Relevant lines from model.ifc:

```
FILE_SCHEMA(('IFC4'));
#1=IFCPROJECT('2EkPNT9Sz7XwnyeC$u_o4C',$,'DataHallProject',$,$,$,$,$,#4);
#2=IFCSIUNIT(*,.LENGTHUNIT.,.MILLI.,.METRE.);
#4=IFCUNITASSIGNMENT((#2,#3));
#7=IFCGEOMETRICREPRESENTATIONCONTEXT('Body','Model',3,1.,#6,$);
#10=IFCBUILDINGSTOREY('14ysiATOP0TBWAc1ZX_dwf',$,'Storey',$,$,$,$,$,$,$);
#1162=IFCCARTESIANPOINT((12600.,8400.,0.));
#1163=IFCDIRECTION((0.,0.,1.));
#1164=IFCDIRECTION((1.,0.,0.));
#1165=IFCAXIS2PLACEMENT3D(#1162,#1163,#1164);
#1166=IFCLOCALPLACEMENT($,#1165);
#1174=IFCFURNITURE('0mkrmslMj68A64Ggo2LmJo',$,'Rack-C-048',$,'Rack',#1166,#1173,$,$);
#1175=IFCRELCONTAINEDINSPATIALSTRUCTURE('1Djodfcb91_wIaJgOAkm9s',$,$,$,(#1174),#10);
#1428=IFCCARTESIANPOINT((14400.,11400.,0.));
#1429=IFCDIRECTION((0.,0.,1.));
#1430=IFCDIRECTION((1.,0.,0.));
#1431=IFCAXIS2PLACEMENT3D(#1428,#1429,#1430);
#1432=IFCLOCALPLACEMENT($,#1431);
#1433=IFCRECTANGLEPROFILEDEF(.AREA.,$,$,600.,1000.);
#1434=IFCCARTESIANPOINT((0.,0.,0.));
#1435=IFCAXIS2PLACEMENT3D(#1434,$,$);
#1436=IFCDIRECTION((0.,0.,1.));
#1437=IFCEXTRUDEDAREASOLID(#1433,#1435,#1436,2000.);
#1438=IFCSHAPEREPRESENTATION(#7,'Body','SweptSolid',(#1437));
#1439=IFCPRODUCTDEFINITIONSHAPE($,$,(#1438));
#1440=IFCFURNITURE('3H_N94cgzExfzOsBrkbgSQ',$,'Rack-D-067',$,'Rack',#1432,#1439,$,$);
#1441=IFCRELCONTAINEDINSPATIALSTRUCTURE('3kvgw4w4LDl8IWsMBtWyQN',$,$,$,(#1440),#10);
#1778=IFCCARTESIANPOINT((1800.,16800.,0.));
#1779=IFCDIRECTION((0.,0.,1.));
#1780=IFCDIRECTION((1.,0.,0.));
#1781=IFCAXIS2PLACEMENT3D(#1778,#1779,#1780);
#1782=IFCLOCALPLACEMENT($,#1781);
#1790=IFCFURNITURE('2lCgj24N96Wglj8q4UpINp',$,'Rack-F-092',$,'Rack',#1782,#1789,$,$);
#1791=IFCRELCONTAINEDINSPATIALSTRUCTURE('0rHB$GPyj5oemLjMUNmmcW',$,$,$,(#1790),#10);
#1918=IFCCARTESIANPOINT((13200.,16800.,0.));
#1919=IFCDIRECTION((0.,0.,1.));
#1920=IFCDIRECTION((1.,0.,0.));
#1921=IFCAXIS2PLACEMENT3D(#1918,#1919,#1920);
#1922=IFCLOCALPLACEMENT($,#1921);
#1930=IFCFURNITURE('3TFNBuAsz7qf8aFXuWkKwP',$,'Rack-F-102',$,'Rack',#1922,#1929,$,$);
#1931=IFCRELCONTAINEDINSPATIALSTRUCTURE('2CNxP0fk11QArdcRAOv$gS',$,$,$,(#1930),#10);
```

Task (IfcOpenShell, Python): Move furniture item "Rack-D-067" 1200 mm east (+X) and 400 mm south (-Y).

```python
import ifcopenshell
import ifcopenshell.api.geometry
import ifcopenshell.util.placement
import ifcopenshell.util.unit

model = ifcopenshell.open("model.ifc")
unit_scale = ifcopenshell.util.unit.calculate_unit_scale(model)

item = model.by_id(1440)
matrix = ifcopenshell.util.placement.get_local_placement(item.ObjectPlacement)
matrix[0, 3] += 1.2 / unit_scale
matrix[1, 3] -= 0.4 / unit_scale
ifcopenshell.api.geometry.edit_object_placement(model, product=item, matrix=matrix, is_si=False)

print(ifcopenshell.util.placement.get_local_placement(item.ObjectPlacement).round(3) + 0.0)

model.write("model_updated.ifc")
```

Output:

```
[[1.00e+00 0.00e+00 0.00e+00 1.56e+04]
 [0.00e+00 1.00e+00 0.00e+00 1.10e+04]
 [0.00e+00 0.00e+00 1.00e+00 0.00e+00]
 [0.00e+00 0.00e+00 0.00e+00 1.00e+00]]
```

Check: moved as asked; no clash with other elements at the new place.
